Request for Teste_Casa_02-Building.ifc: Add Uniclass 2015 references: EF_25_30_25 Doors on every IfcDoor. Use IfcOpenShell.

First a look at what the model holds.

```python
import ifcopenshell

model = ifcopenshell.open("Teste_Casa_02-Building.ifc")
print(model.schema)
print("classifications:", [c.Name for c in model.by_type("IfcClassification")])
for ifc_class in ("IfcDoor", "IfcRoof", "IfcStair", "IfcWall", "IfcWindow"):
    print(ifc_class, len(model.by_type(ifc_class)))
```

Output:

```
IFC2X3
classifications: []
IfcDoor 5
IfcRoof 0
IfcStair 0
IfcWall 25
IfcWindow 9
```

```python
import ifcopenshell
import ifcopenshell.api.classification

model = ifcopenshell.open("Teste_Casa_02-Building.ifc")

# IFC2X3 requires Source and Edition and has no link from the project to the system.
system = model.create_entity("IfcClassification", Source="NBS", Edition="2015", Name="Uniclass 2015")

codes = {
    "IfcDoor": ("EF_25_30_25", "Doors"),
}
for ifc_class, (code, name) in codes.items():
    products = model.by_type(ifc_class)
    ifcopenshell.api.classification.add_reference(
        model, products=products, classification=system, identification=code, name=name
    )
    print(code, len(products))

model.write("Teste_Casa_02-Building_edited.ifc")
```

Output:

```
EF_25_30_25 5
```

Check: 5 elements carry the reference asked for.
